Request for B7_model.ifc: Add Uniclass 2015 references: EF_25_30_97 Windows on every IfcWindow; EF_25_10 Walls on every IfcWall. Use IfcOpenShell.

First a look at what the model holds.

```python
import ifcopenshell

model = ifcopenshell.open("B7_model.ifc")
print(model.schema)
print("classifications:", [c.Name for c in model.by_type("IfcClassification")])
for ifc_class in ("IfcDoor", "IfcRoof", "IfcStair", "IfcWall", "IfcWindow"):
    print(ifc_class, len(model.by_type(ifc_class)))
```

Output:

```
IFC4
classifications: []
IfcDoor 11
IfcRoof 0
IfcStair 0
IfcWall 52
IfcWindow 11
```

```python
import ifcopenshell
import ifcopenshell.api.classification

model = ifcopenshell.open("B7_model.ifc")

system = ifcopenshell.api.classification.add_classification(model, classification="Uniclass 2015")

codes = {
    "IfcWindow": ("EF_25_30_97", "Windows"),
    "IfcWall": ("EF_25_10", "Walls"),
}
for ifc_class, (code, name) in codes.items():
    products = model.by_type(ifc_class)
    ifcopenshell.api.classification.add_reference(
        model, products=products, classification=system, identification=code, name=name
    )
    print(code, len(products))

model.write("B7_model_rev.ifc")
```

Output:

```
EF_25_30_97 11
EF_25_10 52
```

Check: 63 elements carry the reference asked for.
